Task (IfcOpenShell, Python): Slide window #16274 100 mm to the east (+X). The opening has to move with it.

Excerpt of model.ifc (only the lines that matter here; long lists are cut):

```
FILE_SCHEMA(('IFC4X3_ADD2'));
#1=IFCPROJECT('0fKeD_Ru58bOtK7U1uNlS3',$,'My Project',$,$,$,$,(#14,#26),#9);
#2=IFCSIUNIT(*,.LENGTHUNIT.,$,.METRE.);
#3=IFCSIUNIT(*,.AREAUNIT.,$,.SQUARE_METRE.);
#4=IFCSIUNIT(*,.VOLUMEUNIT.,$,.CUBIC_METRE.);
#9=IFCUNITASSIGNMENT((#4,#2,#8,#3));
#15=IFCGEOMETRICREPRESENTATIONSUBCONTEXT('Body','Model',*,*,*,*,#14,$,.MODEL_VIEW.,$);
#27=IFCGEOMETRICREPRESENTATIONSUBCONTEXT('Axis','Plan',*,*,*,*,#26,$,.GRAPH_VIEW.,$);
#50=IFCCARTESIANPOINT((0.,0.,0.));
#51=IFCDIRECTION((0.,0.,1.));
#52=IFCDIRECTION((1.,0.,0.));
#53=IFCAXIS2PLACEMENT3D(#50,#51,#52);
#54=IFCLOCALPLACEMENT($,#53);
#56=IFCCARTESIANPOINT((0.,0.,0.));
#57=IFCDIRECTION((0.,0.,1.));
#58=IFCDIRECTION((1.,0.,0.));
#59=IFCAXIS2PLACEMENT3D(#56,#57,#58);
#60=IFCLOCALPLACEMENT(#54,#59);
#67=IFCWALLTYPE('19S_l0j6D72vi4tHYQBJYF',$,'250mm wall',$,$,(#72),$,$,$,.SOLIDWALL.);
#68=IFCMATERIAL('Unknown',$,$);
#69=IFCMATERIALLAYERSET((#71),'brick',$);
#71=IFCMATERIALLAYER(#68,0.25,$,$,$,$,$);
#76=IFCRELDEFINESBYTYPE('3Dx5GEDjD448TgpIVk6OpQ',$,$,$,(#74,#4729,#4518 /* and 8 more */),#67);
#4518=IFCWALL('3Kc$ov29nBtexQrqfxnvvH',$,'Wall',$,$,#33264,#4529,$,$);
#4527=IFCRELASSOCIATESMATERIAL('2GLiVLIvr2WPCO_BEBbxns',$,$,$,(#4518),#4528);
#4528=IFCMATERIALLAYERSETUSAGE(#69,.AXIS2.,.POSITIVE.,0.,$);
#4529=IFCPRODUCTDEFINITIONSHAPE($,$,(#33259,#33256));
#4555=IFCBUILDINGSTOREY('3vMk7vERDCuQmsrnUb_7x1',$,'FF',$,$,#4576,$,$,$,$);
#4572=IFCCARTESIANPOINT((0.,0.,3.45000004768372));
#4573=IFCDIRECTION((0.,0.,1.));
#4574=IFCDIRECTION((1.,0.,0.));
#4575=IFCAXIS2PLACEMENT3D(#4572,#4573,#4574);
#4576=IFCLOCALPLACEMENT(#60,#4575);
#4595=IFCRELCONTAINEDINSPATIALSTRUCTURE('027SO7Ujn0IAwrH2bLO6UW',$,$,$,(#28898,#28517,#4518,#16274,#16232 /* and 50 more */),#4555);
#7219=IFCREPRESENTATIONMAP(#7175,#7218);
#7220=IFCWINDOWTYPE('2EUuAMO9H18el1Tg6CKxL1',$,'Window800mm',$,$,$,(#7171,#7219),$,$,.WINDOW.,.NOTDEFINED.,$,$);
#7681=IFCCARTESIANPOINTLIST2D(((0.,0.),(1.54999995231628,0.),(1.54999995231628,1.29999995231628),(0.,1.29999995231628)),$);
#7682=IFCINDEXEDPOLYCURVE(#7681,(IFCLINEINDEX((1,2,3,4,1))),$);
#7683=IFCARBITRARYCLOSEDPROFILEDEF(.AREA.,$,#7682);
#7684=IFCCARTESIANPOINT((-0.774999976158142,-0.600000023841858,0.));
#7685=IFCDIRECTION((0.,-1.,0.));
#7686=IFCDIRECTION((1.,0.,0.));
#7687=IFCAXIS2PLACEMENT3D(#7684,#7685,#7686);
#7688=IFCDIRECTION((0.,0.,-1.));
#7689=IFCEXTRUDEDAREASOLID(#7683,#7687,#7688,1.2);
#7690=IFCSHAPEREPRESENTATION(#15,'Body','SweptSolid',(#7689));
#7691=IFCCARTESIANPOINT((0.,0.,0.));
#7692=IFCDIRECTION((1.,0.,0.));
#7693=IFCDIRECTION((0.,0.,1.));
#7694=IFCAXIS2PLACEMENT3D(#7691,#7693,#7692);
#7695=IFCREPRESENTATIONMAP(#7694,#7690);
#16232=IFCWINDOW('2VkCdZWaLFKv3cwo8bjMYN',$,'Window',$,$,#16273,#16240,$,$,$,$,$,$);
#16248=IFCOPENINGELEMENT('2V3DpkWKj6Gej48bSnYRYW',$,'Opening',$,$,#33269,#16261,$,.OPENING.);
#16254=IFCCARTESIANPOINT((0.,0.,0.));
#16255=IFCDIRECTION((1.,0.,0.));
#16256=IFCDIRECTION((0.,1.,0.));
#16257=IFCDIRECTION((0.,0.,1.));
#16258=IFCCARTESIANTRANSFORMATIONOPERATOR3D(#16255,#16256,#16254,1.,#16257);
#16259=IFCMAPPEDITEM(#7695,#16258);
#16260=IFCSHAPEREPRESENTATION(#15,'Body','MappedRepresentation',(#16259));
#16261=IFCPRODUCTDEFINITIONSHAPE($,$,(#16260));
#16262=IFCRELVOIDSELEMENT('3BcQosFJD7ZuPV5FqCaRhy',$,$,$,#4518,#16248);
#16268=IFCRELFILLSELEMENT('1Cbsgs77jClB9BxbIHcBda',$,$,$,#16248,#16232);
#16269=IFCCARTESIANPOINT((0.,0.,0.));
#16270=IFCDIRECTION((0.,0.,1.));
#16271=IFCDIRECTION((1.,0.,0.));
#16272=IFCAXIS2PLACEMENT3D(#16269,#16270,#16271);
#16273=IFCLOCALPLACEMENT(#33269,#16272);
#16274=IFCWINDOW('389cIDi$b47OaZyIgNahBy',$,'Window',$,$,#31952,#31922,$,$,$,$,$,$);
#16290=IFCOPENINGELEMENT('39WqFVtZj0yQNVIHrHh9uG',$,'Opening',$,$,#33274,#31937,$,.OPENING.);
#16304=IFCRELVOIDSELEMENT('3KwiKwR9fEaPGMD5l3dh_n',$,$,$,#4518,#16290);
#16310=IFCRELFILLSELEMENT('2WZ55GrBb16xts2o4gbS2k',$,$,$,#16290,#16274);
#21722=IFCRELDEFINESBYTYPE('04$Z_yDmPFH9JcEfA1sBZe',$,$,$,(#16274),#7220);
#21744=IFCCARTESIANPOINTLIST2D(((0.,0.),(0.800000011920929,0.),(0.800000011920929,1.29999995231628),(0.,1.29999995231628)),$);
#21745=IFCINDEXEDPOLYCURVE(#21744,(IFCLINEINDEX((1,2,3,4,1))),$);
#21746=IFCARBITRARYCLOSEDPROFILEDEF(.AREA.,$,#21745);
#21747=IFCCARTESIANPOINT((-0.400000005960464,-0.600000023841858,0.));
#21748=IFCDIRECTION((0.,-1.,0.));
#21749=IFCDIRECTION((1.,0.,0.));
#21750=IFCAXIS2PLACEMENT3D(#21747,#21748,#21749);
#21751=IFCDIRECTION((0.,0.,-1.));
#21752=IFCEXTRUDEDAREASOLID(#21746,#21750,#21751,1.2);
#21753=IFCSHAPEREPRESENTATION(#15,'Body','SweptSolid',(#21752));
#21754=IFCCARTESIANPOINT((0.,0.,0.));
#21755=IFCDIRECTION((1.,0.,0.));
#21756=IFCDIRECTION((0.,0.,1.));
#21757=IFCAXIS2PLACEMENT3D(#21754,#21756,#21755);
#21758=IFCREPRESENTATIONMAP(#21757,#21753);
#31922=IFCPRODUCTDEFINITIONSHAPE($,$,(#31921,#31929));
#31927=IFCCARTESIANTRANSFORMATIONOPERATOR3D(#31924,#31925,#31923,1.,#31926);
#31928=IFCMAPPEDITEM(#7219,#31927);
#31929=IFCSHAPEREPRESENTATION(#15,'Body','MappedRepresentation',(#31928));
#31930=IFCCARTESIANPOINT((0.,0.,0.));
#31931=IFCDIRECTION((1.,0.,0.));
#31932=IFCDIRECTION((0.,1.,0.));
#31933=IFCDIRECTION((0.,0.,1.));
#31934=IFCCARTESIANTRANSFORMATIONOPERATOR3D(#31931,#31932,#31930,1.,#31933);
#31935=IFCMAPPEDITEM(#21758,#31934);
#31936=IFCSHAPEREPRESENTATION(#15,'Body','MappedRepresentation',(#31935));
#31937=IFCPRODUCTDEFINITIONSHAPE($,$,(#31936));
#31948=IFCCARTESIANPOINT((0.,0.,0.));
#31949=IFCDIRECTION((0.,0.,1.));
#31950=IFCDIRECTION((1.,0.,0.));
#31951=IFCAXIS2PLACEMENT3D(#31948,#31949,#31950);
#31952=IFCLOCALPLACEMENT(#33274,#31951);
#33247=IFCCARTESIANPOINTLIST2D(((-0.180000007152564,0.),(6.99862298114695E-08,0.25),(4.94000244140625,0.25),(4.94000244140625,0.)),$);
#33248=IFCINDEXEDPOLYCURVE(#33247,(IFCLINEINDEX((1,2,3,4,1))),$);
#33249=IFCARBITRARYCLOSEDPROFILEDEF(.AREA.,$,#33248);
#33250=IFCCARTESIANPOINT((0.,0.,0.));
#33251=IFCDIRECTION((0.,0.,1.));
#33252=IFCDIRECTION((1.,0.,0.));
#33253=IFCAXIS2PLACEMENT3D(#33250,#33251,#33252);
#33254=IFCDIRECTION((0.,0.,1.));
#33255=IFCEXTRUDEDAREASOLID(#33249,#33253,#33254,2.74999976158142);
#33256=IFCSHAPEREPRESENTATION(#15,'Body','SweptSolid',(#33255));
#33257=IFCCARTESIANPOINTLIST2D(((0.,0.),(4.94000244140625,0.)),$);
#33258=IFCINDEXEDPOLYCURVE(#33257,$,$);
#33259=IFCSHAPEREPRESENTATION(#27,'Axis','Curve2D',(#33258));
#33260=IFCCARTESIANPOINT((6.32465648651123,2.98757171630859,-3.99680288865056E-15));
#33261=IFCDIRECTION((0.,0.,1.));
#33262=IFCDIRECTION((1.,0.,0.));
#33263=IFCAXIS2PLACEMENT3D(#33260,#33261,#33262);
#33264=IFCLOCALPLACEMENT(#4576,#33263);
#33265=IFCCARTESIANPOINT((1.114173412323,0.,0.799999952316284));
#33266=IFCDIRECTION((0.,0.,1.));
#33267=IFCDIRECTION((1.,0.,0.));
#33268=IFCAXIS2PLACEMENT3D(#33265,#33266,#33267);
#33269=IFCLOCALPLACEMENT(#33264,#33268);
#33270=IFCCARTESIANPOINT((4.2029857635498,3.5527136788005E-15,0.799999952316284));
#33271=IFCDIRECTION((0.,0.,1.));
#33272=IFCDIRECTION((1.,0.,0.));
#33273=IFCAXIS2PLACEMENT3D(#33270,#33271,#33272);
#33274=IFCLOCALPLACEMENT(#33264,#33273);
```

```python
import ifcopenshell
import ifcopenshell.api.geometry
import ifcopenshell.util.placement
import ifcopenshell.util.unit

model = ifcopenshell.open("model.ifc")
unit_scale = ifcopenshell.util.unit.calculate_unit_scale(model)

window = model.by_id(16274)
opening = window.FillsVoids[0].RelatingOpeningElement
wall = opening.VoidsElements[0].RelatingBuildingElement

wall_matrix = ifcopenshell.util.placement.get_local_placement(wall.ObjectPlacement)
shift = wall_matrix[:3, 0] * 0.1 / unit_scale
before = ifcopenshell.util.placement.get_local_placement(window.ObjectPlacement)[:3, 3].copy()

# The window is placed relative to its opening, so it follows when the opening moves.
matrix = ifcopenshell.util.placement.get_local_placement(opening.ObjectPlacement)
matrix[:3, 3] += shift
ifcopenshell.api.geometry.edit_object_placement(
    model, product=opening, matrix=matrix, is_si=False, should_transform_children=True
)

after = ifcopenshell.util.placement.get_local_placement(window.ObjectPlacement)[:3, 3]
print("window moved by", (after - before).round(3) + 0.0)

model.write("model_rev.ifc")
```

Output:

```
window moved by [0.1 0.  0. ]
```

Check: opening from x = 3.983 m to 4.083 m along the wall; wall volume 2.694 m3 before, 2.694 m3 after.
